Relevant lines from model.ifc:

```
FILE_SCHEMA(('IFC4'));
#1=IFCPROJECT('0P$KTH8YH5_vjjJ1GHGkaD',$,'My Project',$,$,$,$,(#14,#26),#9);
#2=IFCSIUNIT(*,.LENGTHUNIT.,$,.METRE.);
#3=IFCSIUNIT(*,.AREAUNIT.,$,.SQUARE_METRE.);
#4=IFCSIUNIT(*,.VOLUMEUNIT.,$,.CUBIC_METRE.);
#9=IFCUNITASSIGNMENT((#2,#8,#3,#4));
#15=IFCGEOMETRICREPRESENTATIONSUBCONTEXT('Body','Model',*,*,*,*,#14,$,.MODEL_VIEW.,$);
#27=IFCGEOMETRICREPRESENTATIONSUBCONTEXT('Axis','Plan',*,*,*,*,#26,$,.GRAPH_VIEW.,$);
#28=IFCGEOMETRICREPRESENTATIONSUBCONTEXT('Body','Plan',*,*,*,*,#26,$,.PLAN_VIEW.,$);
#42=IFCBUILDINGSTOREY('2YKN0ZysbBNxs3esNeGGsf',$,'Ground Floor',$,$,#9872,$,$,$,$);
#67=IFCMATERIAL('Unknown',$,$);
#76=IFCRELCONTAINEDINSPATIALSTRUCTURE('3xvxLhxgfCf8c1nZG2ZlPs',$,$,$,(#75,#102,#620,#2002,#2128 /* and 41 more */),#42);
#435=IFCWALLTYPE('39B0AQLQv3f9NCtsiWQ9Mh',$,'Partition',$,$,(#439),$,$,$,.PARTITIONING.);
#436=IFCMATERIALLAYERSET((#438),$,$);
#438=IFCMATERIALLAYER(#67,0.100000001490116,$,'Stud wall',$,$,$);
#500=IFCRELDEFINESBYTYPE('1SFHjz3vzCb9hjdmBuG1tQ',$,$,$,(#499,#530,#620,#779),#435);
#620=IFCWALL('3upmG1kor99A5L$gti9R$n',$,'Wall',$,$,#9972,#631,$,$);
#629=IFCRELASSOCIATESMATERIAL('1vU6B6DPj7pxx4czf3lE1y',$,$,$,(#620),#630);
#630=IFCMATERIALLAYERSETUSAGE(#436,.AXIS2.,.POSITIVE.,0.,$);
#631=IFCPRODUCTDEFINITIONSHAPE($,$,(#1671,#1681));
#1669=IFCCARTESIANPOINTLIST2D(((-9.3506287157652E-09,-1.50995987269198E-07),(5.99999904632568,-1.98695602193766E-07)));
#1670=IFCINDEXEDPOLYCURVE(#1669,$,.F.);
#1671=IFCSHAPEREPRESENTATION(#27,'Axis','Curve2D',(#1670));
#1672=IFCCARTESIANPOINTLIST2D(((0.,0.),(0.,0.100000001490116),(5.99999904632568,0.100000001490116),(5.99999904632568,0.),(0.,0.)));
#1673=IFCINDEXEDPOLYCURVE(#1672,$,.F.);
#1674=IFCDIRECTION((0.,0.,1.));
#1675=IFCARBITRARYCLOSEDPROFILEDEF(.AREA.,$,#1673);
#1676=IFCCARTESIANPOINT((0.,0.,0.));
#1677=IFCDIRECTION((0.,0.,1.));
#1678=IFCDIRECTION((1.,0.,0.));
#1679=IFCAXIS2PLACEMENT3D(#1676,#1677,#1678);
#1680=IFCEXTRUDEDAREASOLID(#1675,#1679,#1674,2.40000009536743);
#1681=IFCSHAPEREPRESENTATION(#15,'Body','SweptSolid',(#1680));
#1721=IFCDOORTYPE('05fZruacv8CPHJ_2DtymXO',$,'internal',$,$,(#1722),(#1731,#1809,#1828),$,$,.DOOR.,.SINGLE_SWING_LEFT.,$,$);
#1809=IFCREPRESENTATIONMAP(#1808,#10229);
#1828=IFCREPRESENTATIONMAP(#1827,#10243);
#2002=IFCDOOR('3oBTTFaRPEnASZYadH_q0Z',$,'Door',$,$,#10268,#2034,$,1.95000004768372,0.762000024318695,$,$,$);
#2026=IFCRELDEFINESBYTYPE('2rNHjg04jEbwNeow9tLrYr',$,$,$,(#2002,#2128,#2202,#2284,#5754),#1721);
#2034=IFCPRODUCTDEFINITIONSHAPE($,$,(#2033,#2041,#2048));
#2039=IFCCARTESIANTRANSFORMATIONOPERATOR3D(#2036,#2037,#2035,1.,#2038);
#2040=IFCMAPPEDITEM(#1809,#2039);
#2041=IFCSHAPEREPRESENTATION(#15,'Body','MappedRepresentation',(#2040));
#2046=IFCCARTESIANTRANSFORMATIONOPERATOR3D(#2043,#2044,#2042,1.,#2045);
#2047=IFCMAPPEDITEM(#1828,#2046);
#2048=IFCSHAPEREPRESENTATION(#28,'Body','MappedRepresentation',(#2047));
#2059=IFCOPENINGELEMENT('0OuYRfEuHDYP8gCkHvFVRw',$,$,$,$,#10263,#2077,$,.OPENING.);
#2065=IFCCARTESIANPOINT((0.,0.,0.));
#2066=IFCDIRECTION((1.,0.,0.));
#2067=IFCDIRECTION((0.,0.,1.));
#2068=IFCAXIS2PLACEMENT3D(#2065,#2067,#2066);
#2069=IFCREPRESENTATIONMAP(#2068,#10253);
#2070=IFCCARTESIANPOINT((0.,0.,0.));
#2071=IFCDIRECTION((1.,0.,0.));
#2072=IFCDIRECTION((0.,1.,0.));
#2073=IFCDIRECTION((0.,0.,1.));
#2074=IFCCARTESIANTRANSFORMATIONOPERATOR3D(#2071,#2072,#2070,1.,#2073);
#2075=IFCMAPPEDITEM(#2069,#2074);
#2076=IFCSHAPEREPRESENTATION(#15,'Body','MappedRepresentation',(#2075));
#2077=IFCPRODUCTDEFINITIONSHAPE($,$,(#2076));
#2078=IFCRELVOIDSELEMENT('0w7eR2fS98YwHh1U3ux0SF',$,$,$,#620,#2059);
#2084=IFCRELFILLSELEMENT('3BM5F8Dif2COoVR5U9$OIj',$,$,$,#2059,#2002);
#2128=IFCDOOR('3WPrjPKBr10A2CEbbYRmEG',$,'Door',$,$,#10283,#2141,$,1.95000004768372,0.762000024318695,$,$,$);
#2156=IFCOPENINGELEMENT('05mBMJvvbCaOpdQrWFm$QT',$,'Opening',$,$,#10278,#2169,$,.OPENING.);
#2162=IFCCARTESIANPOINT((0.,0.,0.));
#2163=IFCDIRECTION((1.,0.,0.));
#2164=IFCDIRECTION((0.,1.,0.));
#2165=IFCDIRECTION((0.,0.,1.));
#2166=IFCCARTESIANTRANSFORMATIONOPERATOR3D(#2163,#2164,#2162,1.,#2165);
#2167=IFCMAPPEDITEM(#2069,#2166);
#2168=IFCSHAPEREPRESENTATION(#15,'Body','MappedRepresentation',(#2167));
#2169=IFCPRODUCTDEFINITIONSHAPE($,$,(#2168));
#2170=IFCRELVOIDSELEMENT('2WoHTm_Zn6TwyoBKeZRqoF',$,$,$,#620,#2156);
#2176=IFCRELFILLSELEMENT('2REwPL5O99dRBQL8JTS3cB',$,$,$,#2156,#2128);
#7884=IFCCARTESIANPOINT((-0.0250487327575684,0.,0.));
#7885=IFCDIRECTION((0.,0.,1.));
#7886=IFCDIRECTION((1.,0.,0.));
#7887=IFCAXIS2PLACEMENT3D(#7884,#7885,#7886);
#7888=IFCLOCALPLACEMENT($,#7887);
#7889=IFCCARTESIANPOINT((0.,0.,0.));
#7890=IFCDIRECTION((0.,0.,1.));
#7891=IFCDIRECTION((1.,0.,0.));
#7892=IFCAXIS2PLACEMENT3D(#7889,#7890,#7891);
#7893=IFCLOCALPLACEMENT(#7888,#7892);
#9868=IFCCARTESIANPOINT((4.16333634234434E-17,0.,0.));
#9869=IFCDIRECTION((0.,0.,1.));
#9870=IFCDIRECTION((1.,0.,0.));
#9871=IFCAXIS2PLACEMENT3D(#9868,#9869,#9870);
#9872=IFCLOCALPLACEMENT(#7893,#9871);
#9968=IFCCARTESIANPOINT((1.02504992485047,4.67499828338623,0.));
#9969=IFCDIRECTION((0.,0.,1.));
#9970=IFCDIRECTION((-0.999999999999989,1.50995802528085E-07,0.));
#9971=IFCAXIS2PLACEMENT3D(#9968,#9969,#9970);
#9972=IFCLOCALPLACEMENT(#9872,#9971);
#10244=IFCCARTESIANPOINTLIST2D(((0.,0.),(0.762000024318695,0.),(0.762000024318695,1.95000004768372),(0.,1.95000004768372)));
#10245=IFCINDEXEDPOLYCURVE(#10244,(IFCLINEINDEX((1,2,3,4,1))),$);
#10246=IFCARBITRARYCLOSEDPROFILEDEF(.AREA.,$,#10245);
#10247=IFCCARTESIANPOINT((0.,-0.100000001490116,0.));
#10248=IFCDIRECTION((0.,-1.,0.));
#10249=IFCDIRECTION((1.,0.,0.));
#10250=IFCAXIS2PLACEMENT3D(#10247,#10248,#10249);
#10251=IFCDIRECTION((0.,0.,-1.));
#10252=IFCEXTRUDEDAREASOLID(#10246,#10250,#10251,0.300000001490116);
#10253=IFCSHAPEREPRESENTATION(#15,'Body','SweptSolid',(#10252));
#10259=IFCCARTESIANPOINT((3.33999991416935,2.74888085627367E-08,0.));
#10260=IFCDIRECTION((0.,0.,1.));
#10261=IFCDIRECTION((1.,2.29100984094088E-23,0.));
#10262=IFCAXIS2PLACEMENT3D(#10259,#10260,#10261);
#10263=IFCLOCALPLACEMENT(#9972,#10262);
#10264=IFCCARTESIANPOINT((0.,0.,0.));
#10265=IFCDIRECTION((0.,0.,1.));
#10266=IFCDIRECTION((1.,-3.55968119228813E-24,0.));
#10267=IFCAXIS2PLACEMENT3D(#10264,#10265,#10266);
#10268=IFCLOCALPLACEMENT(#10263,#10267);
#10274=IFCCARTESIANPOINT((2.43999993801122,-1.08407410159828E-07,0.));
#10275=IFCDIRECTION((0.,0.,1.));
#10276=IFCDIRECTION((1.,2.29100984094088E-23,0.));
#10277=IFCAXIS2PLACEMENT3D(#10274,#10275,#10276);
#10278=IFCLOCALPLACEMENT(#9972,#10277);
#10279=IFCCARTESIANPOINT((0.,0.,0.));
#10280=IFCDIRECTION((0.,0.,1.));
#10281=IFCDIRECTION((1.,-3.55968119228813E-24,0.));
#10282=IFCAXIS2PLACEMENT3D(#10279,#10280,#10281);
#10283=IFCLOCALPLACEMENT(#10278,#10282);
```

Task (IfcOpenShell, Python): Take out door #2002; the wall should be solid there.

```python
import ifcopenshell
import ifcopenshell.api.feature
import ifcopenshell.api.root
import ifcopenshell.geom
import ifcopenshell.util.shape

model = ifcopenshell.open("model.ifc")
settings = ifcopenshell.geom.settings()


def volume(element):
    """Net volume in cubic metres, openings subtracted."""
    shape = ifcopenshell.geom.create_shape(settings, element)
    return ifcopenshell.util.shape.get_volume(shape.geometry)


door = model.by_guid("3oBTTFaRPEnASZYadH_q0Z")
opening = door.FillsVoids[0].RelatingOpeningElement
wall = opening.VoidsElements[0].RelatingBuildingElement
before = volume(wall)

ifcopenshell.api.root.remove_product(model, product=door)
ifcopenshell.api.feature.remove_feature(model, feature=opening)

after = volume(wall)

print(f"wall volume {before:.3f} -> {after:.3f} m3")

model.write("model-out.ifc")
```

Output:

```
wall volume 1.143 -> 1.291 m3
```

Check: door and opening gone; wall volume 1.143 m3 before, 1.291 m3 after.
